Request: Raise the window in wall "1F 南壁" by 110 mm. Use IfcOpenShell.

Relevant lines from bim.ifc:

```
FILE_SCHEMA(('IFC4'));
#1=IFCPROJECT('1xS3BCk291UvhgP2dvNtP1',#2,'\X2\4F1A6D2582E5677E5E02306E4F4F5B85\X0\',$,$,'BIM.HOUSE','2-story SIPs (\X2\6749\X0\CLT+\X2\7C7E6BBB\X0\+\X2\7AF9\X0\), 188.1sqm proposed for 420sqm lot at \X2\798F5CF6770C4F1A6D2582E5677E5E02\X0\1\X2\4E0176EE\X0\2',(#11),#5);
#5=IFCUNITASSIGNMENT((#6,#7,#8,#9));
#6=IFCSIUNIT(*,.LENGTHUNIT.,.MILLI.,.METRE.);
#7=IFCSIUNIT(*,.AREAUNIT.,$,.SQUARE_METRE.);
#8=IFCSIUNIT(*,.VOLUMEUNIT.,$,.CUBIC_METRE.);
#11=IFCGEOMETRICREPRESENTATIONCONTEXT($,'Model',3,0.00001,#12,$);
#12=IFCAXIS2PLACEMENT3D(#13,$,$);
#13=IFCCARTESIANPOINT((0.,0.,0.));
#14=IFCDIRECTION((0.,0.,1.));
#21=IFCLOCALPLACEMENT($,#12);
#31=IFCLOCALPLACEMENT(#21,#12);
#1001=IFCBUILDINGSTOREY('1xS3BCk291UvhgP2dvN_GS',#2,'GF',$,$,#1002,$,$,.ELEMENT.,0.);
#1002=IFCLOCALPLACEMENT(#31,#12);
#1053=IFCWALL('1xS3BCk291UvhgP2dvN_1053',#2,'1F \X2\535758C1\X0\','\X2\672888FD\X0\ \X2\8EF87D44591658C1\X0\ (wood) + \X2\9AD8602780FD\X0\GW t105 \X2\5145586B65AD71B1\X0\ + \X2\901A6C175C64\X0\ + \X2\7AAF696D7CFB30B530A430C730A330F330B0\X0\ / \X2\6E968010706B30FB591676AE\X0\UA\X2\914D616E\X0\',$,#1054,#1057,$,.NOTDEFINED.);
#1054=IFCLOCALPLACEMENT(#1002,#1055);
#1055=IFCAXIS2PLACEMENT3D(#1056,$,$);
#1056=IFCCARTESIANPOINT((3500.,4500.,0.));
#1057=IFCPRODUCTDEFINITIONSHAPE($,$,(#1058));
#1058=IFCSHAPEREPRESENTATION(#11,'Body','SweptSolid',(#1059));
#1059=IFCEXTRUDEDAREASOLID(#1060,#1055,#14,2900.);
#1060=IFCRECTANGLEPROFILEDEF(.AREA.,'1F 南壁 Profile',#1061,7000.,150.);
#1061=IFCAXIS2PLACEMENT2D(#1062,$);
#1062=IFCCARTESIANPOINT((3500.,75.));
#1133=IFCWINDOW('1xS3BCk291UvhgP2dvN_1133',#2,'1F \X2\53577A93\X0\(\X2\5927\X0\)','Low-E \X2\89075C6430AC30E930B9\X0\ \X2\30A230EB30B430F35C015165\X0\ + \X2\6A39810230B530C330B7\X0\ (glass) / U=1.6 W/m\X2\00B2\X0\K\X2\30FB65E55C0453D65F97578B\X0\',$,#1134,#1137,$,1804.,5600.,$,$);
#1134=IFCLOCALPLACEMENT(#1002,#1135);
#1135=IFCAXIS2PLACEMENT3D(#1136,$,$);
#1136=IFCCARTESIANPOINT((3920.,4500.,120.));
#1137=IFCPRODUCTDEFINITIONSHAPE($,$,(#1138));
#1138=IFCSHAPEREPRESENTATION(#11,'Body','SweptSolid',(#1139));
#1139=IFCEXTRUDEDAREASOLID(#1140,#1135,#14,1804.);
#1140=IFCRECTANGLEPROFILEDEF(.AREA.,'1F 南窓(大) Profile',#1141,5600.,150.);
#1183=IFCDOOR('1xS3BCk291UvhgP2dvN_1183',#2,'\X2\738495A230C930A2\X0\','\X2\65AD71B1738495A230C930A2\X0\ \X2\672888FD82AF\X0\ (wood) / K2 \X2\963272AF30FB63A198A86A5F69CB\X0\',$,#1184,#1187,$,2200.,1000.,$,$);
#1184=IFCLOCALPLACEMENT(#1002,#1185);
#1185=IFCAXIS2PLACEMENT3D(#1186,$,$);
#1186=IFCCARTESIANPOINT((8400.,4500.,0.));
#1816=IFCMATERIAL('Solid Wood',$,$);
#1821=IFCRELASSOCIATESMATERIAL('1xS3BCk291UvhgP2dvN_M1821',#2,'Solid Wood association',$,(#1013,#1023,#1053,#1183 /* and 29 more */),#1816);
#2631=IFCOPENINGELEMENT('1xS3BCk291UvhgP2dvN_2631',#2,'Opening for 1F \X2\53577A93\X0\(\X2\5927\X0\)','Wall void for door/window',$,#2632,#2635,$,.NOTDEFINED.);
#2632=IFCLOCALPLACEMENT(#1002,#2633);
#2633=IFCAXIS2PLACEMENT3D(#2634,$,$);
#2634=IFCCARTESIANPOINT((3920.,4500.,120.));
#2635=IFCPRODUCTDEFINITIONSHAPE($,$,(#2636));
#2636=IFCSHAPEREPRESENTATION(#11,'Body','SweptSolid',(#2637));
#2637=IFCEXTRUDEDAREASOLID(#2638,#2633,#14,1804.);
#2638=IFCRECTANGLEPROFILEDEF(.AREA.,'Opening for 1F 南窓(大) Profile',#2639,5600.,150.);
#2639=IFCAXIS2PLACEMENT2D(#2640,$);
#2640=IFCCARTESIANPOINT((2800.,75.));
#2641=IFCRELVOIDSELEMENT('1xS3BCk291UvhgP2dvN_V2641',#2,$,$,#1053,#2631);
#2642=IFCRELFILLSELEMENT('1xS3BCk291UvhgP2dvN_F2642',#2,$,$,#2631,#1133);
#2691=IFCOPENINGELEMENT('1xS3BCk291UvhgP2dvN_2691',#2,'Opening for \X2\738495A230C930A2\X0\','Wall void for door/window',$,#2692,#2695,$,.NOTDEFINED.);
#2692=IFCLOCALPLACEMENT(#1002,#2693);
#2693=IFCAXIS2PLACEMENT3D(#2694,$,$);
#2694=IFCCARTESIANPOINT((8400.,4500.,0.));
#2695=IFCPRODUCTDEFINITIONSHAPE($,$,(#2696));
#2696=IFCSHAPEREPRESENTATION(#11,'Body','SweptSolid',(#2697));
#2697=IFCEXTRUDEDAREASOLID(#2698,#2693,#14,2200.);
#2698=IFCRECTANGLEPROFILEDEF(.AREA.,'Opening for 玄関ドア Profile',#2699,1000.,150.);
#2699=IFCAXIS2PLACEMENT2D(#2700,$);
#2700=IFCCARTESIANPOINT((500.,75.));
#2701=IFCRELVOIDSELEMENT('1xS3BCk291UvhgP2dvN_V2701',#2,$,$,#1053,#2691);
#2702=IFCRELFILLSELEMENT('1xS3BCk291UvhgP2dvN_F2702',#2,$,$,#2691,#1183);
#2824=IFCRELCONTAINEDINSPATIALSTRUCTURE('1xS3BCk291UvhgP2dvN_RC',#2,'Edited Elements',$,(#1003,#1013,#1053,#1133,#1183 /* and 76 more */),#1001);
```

```python
import numpy as np
import ifcopenshell
import ifcopenshell.api.geometry
import ifcopenshell.util.placement
import ifcopenshell.util.unit

model = ifcopenshell.open("bim.ifc")
unit_scale = ifcopenshell.util.unit.calculate_unit_scale(model)

window = model.by_guid("1xS3BCk291UvhgP2dvN_1133")
opening = window.FillsVoids[0].RelatingOpeningElement
dz = 110.0

shift = np.array([0.0, 0.0, dz])
# The window is not placed relative to its opening, so move both.
for product in (opening, window):
    matrix = ifcopenshell.util.placement.get_local_placement(product.ObjectPlacement)
    matrix[:3, 3] += shift
    ifcopenshell.api.geometry.edit_object_placement(model, product=product, matrix=matrix, is_si=False)

print(f"moved by {dz * unit_scale:+.3f} m")

model.write("bim_edited.ifc")
```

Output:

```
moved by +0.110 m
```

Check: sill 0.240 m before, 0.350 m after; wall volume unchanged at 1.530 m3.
